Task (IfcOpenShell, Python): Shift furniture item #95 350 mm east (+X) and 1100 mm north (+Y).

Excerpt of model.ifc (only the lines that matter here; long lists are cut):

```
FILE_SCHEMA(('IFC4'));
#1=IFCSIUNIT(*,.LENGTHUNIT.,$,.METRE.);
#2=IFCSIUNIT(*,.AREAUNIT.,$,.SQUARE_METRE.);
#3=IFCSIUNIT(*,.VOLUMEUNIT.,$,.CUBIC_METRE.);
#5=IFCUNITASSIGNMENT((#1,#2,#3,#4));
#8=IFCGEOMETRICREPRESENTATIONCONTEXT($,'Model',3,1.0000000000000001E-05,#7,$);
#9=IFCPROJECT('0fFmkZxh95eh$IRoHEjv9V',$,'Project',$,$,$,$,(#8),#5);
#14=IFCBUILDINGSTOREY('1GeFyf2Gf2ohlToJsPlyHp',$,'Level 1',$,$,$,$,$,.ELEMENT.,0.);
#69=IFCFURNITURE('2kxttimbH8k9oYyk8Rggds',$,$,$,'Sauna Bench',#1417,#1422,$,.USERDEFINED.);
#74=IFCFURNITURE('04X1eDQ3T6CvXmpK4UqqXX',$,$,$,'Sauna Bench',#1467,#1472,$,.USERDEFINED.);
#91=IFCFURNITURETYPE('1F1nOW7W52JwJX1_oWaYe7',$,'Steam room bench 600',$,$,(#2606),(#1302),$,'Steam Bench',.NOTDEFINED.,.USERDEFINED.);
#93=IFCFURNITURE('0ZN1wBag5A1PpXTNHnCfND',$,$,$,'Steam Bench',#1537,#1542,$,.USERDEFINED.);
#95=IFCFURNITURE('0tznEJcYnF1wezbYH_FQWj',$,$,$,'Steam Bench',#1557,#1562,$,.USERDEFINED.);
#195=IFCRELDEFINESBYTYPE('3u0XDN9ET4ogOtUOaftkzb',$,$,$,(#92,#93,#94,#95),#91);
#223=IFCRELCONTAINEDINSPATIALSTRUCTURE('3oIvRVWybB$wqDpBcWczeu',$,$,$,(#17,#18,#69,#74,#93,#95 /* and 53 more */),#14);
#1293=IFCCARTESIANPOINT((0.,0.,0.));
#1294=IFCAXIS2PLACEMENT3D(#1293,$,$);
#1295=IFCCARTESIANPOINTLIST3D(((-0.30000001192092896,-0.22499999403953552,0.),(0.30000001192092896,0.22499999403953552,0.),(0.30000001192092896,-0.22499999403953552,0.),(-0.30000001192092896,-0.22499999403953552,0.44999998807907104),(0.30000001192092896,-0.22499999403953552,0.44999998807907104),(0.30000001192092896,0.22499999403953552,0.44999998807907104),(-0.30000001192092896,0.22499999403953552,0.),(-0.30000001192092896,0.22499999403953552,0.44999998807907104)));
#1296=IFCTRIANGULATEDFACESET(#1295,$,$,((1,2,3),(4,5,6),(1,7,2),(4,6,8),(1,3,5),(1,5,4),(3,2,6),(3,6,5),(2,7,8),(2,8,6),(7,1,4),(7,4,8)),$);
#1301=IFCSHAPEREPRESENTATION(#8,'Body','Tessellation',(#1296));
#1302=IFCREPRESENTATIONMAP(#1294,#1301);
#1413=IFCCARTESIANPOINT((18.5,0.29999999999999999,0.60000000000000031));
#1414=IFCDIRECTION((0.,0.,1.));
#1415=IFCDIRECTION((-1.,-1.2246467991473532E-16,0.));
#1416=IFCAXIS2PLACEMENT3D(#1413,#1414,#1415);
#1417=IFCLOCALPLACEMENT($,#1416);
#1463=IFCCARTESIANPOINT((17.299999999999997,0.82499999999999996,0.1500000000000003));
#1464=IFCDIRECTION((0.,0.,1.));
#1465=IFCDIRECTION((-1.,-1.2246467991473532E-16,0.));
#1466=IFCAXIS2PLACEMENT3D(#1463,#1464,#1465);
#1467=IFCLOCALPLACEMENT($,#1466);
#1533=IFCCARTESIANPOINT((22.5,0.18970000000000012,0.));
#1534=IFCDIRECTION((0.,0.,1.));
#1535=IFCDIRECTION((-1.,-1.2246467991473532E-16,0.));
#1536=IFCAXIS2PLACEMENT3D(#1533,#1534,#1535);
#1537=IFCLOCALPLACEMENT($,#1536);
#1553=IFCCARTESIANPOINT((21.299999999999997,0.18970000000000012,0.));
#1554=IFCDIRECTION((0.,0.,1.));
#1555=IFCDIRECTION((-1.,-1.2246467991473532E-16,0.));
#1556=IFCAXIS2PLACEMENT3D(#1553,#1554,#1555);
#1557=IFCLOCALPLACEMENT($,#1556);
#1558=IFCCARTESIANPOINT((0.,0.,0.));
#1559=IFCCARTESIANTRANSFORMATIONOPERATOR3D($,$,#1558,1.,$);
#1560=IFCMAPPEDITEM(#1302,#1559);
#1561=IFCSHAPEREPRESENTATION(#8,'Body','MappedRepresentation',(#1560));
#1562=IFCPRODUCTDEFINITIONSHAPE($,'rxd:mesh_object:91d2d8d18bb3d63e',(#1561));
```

```python
import ifcopenshell
import ifcopenshell.api.geometry
import ifcopenshell.util.placement

model = ifcopenshell.open("model.ifc")

item = model.by_guid("0tznEJcYnF1wezbYH_FQWj")
matrix = ifcopenshell.util.placement.get_local_placement(item.ObjectPlacement)
matrix[0, 3] += 0.35
matrix[1, 3] += 1.1
ifcopenshell.api.geometry.edit_object_placement(model, product=item, matrix=matrix, is_si=False)

print(ifcopenshell.util.placement.get_local_placement(item.ObjectPlacement).round(3) + 0.0)

model.write("model_v2.ifc")
```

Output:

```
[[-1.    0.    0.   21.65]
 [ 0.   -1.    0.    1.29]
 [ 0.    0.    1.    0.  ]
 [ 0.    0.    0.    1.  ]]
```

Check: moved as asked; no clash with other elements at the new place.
